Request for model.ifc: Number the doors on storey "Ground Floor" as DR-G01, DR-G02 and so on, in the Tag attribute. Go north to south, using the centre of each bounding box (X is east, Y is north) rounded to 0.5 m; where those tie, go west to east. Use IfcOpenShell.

First a look at what the model holds.

```python
import ifcopenshell
import ifcopenshell.util.element
import ifcopenshell.util.placement

model = ifcopenshell.open("model.ifc")
print(model.schema)
storey = next(s for s in model.by_type("IfcBuildingStorey") if s.Name == "Ground Floor")
doors = [e for e in ifcopenshell.util.element.get_decomposition(storey) if e.is_a("IfcDoor")]
for e in sorted(doors, key=lambda e: e.id()):
    origin = ifcopenshell.util.placement.get_local_placement(e.ObjectPlacement)[:3, 3]
    print(e.id(), e.Tag, e.Name, origin.round(2) + 0.0, sep=" | ")
```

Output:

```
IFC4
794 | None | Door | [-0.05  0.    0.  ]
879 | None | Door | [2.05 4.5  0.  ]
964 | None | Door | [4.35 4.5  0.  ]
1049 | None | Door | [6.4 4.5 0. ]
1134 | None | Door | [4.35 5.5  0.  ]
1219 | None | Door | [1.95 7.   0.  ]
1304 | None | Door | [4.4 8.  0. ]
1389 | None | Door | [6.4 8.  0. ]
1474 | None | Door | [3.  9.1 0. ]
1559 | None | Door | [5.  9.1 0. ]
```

```python
import ifcopenshell
import ifcopenshell.geom
import ifcopenshell.util.element
import ifcopenshell.util.shape

model = ifcopenshell.open("model.ifc")
settings = ifcopenshell.geom.settings()
settings.set("use-world-coords", True)


def centre(element):
    shape = ifcopenshell.geom.create_shape(settings, element)
    return ifcopenshell.util.shape.get_bbox_centroid(shape.geometry)


storey = next(s for s in model.by_type("IfcBuildingStorey") if s.Name == "Ground Floor")
doors = [e for e in ifcopenshell.util.element.get_decomposition(storey) if e.is_a("IfcDoor")]

# Insertion points can sit at a corner or the storey origin, so sort by the geometry (in metres).
centres = {e: centre(e) for e in doors}
doors.sort(key=lambda e: (-round(centres[e][1] / 0.5), centres[e][0]))

for i, e in enumerate(doors, start=1):
    number = f"DR-G{i:02d}"
    e.Tag = number
    print(e.id(), number)

model.write("model_v2.ifc")
```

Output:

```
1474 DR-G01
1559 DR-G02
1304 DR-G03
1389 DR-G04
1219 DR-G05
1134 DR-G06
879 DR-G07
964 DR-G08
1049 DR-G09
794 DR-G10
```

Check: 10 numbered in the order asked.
